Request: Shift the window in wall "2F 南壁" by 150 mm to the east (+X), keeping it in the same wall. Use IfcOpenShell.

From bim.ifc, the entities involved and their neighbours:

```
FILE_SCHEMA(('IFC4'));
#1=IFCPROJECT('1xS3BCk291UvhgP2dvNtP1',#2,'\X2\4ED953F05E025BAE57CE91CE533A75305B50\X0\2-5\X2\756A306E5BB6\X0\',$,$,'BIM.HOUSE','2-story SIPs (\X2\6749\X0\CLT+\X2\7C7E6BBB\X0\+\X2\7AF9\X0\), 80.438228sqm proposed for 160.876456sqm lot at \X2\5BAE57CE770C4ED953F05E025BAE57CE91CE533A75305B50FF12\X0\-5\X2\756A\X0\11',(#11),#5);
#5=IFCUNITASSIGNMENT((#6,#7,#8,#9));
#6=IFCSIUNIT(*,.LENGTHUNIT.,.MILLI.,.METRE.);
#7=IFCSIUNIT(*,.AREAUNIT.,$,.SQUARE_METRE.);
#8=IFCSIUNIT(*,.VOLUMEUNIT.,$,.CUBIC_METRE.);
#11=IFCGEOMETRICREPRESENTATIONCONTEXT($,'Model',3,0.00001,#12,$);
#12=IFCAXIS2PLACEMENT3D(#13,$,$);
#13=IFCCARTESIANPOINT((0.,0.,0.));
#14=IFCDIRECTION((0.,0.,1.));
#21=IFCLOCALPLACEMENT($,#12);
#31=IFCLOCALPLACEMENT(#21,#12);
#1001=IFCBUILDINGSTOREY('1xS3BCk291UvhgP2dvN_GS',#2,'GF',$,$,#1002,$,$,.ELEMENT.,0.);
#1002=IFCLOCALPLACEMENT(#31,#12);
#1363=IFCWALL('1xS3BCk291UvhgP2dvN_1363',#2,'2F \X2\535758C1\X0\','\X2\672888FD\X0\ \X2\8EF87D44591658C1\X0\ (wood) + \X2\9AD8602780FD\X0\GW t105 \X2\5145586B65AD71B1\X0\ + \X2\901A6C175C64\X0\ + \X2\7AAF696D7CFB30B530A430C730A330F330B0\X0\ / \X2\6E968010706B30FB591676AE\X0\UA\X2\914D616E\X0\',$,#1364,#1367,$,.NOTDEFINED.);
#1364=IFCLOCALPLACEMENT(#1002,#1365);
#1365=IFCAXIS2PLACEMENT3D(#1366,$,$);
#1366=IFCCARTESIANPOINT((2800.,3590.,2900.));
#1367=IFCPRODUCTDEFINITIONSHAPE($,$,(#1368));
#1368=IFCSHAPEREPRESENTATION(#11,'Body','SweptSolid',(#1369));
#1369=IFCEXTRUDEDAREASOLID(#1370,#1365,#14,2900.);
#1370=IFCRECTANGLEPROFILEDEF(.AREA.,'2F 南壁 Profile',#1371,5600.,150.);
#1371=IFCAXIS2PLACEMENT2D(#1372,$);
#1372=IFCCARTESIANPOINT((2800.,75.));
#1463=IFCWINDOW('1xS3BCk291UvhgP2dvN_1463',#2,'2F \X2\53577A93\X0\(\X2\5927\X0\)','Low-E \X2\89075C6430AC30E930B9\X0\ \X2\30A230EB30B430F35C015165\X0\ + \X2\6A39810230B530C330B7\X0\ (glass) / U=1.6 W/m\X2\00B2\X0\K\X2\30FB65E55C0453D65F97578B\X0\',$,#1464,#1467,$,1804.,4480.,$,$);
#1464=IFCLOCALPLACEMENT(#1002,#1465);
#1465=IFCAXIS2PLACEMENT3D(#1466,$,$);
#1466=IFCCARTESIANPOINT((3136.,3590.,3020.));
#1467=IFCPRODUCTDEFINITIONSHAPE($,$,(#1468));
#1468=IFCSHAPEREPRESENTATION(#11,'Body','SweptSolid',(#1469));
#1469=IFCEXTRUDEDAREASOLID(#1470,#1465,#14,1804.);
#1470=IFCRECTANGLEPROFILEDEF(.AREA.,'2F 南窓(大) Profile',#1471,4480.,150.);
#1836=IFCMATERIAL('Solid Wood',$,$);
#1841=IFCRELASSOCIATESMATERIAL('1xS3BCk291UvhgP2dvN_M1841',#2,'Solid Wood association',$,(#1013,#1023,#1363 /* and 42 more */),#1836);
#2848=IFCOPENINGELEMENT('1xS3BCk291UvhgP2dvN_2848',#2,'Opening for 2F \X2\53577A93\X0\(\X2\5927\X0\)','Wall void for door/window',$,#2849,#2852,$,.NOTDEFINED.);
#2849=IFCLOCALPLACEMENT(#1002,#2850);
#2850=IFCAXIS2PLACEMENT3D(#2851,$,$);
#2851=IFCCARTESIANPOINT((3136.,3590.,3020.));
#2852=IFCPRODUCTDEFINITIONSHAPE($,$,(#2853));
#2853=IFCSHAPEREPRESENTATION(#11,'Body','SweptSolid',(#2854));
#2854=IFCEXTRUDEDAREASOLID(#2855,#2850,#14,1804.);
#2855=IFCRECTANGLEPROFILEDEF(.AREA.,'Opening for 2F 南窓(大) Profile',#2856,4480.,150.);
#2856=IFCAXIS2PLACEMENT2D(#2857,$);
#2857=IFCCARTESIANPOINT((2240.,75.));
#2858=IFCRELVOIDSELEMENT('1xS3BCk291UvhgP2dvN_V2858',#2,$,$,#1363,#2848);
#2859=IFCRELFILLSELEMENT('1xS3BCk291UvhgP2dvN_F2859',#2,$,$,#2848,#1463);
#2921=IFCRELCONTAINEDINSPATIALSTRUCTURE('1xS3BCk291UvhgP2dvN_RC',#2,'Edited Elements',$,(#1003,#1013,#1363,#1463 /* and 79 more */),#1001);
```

```python
import ifcopenshell
import ifcopenshell.api.geometry
import ifcopenshell.util.placement
import ifcopenshell.util.unit

model = ifcopenshell.open("bim.ifc")
unit_scale = ifcopenshell.util.unit.calculate_unit_scale(model)

window = model.by_id(1463)
opening = window.FillsVoids[0].RelatingOpeningElement
wall = opening.VoidsElements[0].RelatingBuildingElement

wall_matrix = ifcopenshell.util.placement.get_local_placement(wall.ObjectPlacement)
shift = wall_matrix[:3, 0] * 0.15 / unit_scale
before = ifcopenshell.util.placement.get_local_placement(window.ObjectPlacement)[:3, 3].copy()

# The window is not placed relative to its opening, so move both.
for product in (opening, window):
    matrix = ifcopenshell.util.placement.get_local_placement(product.ObjectPlacement)
    matrix[:3, 3] += shift
    ifcopenshell.api.geometry.edit_object_placement(model, product=product, matrix=matrix, is_si=False)

after = ifcopenshell.util.placement.get_local_placement(window.ObjectPlacement)[:3, 3]
print("window moved by", (after - before).round(3) + 0.0)

model.write("bim_updated.ifc")
```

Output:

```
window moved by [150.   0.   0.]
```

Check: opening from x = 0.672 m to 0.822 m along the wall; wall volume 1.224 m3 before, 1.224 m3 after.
